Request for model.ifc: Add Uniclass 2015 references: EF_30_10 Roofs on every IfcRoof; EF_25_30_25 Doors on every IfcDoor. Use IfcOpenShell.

First a look at what the model holds.

```python
import ifcopenshell

model = ifcopenshell.open("model.ifc")
print(model.schema)
print("classifications:", [c.Name for c in model.by_type("IfcClassification")])
for ifc_class in ("IfcDoor", "IfcRoof", "IfcStair", "IfcWall", "IfcWindow"):
    print(ifc_class, len(model.by_type(ifc_class)))
```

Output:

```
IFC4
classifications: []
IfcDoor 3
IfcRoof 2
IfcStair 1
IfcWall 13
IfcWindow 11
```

```python
import ifcopenshell
import ifcopenshell.api.classification

model = ifcopenshell.open("model.ifc")

system = ifcopenshell.api.classification.add_classification(model, classification="Uniclass 2015")

codes = {
    "IfcRoof": ("EF_30_10", "Roofs"),
    "IfcDoor": ("EF_25_30_25", "Doors"),
}
for ifc_class, (code, name) in codes.items():
    products = model.by_type(ifc_class)
    ifcopenshell.api.classification.add_reference(
        model, products=products, classification=system, identification=code, name=name
    )
    print(code, len(products))

model.write("model_rev.ifc")
```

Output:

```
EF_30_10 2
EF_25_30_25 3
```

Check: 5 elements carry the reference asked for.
